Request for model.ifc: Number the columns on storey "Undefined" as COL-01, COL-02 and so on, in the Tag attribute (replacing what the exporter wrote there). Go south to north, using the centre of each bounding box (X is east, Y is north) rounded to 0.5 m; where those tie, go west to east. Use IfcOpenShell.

First a look at what the model holds.

```python
import ifcopenshell
import ifcopenshell.util.element
import ifcopenshell.util.placement

model = ifcopenshell.open("model.ifc")
print(model.schema)
storey = next(s for s in model.by_type("IfcBuildingStorey") if s.Name == "Undefined")
columns = [e for e in ifcopenshell.util.element.get_decomposition(storey) if e.is_a("IfcColumn")]
for e in sorted(columns, key=lambda e: e.id()):
    origin = ifcopenshell.util.placement.get_local_placement(e.ObjectPlacement)[:3, 3]
    print(e.id(), e.Tag, e.Name, origin.round(2) + 0.0, sep=" | ")
```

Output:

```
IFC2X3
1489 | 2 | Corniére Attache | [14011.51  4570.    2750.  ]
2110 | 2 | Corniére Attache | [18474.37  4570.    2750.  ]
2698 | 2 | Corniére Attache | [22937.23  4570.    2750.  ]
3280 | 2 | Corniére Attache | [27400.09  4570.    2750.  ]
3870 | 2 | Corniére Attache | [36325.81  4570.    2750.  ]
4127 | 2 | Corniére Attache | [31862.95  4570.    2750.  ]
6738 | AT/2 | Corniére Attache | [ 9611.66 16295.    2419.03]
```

```python
import ifcopenshell
import ifcopenshell.geom
import ifcopenshell.util.element
import ifcopenshell.util.shape

model = ifcopenshell.open("model.ifc")
settings = ifcopenshell.geom.settings()
settings.set("use-world-coords", True)


def centre(element):
    shape = ifcopenshell.geom.create_shape(settings, element)
    return ifcopenshell.util.shape.get_bbox_centroid(shape.geometry)


storey = next(s for s in model.by_type("IfcBuildingStorey") if s.Name == "Undefined")
columns = [e for e in ifcopenshell.util.element.get_decomposition(storey) if e.is_a("IfcColumn")]

# Insertion points can sit at a corner or the storey origin, so sort by the geometry (in metres).
centres = {e: centre(e) for e in columns}
columns.sort(key=lambda e: (round(centres[e][1] / 0.5), centres[e][0]))

for i, e in enumerate(columns, start=1):
    number = f"COL-{i:02d}"
    e.Tag = number
    print(e.id(), number)

model.write("model-out.ifc")
```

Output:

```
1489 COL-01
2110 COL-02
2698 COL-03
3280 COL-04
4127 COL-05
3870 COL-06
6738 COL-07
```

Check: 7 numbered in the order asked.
